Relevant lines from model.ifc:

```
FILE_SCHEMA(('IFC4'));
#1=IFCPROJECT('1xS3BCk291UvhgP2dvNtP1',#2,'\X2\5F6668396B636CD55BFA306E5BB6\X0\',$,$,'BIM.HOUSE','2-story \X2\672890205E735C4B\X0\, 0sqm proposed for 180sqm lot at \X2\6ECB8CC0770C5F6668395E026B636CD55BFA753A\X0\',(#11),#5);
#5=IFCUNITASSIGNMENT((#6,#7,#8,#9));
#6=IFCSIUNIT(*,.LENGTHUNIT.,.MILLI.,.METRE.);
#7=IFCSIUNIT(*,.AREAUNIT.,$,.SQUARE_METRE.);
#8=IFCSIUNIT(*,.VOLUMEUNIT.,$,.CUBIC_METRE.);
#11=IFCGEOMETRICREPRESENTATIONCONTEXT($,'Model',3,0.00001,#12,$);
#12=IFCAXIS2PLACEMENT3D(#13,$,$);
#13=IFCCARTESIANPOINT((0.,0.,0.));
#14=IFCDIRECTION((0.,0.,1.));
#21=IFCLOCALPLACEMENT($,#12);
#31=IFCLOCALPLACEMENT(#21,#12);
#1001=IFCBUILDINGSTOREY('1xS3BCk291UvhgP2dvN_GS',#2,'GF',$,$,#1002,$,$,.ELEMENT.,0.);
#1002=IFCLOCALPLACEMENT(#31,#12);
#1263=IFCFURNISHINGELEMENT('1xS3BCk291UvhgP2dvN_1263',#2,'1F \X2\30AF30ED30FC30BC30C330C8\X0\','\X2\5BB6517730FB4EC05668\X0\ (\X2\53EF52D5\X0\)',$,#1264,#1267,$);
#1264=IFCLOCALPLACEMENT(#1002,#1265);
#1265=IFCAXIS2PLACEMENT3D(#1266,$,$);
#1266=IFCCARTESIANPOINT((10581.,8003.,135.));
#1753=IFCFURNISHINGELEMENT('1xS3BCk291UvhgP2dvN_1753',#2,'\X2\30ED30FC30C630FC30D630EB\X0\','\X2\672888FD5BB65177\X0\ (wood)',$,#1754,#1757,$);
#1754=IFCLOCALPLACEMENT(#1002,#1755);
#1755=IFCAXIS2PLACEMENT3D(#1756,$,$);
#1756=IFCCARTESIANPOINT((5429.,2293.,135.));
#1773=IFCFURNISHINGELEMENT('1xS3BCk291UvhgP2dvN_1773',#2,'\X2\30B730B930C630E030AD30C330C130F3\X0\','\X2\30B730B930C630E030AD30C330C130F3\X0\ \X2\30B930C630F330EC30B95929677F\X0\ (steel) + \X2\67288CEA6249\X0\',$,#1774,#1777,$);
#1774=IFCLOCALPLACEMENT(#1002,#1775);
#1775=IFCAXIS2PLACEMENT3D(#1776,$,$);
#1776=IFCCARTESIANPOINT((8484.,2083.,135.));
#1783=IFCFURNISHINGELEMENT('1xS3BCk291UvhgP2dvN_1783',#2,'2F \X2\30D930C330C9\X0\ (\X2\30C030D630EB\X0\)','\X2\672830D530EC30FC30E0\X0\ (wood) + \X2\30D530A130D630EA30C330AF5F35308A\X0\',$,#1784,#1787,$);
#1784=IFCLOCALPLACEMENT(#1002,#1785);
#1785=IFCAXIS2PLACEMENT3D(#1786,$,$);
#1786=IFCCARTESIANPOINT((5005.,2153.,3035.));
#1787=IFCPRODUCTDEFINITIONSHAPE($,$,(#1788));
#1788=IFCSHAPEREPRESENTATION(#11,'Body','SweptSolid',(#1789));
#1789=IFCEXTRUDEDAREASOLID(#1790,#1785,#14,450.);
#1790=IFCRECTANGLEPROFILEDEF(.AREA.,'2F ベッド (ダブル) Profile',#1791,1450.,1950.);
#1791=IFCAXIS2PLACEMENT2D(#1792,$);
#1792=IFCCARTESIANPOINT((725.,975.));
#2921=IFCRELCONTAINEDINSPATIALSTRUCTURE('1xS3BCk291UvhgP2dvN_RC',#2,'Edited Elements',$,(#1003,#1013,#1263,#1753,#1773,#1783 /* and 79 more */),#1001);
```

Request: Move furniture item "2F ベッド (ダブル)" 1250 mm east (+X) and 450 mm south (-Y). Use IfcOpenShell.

```python
import ifcopenshell
import ifcopenshell.api.geometry
import ifcopenshell.util.placement

model = ifcopenshell.open("model.ifc")

item = model.by_guid("1xS3BCk291UvhgP2dvN_1783")
matrix = ifcopenshell.util.placement.get_local_placement(item.ObjectPlacement)
matrix[0, 3] += 1250.0
matrix[1, 3] -= 450.0
ifcopenshell.api.geometry.edit_object_placement(model, product=item, matrix=matrix, is_si=False)

print(ifcopenshell.util.placement.get_local_placement(item.ObjectPlacement).round(3) + 0.0)

model.write("model_edited.ifc")
```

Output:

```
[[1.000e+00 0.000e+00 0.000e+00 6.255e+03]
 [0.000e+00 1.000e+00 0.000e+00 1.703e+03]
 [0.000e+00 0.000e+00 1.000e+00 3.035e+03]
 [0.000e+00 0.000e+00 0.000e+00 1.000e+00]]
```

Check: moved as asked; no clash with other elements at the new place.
